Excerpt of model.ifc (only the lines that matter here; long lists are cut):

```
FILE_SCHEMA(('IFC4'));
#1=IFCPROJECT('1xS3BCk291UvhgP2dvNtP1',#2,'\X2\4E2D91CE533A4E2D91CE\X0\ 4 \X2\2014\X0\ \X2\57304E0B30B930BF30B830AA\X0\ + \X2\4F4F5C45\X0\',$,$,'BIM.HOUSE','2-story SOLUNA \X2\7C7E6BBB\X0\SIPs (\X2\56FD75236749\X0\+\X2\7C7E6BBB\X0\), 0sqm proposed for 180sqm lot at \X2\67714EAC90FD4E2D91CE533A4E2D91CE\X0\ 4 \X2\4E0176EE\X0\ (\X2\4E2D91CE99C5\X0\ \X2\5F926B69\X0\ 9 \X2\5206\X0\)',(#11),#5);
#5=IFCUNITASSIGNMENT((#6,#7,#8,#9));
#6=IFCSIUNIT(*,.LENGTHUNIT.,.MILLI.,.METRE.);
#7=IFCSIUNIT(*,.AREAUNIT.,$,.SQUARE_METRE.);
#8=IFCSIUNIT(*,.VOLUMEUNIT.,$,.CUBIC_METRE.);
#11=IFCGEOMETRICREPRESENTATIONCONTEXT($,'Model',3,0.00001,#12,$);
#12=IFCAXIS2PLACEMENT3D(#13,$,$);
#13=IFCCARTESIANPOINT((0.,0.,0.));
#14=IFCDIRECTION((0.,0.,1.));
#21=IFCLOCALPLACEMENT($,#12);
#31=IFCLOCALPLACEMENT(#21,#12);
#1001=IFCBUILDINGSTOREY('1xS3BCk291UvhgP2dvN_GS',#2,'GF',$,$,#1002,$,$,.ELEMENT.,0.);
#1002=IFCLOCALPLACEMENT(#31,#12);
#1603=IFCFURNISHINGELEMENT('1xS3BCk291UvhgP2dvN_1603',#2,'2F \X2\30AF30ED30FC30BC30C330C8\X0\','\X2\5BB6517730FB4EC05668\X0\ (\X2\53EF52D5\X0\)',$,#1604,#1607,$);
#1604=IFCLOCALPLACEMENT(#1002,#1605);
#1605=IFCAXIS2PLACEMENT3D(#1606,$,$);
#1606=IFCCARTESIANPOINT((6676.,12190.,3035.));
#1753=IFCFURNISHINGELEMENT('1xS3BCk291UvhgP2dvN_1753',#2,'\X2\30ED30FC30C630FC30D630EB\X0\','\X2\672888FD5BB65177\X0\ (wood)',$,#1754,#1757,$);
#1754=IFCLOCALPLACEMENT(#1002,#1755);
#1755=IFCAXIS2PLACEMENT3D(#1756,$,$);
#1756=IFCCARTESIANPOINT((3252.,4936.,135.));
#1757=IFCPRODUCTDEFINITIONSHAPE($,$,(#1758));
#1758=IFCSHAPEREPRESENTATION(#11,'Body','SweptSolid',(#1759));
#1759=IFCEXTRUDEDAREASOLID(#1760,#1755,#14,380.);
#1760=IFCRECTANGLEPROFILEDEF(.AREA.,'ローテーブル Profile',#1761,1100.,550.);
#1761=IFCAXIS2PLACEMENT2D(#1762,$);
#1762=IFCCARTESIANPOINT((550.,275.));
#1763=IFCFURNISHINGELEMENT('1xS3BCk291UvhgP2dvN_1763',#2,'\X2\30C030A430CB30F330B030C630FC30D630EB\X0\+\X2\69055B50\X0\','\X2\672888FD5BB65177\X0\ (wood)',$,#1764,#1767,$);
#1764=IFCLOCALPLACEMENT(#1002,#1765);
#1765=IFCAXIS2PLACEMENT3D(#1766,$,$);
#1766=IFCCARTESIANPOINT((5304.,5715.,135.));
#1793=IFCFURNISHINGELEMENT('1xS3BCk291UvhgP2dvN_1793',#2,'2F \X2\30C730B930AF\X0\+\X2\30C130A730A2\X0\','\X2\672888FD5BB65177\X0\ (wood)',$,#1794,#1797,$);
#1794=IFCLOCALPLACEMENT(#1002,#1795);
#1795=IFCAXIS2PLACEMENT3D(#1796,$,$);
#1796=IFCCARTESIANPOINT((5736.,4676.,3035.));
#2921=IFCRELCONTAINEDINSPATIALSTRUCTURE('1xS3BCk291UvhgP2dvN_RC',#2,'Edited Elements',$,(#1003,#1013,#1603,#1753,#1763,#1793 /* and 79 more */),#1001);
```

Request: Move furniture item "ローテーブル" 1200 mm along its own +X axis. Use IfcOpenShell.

```python
import ifcopenshell
import ifcopenshell.api.geometry
import ifcopenshell.util.placement
import ifcopenshell.util.unit

model = ifcopenshell.open("model.ifc")
unit_scale = ifcopenshell.util.unit.calculate_unit_scale(model)

item = model.by_guid("1xS3BCk291UvhgP2dvN_1753")
matrix = ifcopenshell.util.placement.get_local_placement(item.ObjectPlacement)
matrix[:3, 3] += matrix[:3, 0] * 1.2 / unit_scale
ifcopenshell.api.geometry.edit_object_placement(model, product=item, matrix=matrix, is_si=False)

print(ifcopenshell.util.placement.get_local_placement(item.ObjectPlacement).round(3) + 0.0)

model.write("model_edited.ifc")
```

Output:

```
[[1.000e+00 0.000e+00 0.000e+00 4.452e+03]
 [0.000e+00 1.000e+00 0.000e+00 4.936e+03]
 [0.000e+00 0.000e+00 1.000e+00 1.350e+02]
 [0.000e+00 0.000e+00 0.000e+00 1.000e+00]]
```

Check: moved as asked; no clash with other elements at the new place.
